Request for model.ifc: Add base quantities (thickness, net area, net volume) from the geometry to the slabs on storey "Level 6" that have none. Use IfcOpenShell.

First a look at what the model holds.

```python
import ifcopenshell
import ifcopenshell.util.element
import ifcopenshell.util.unit

model = ifcopenshell.open("model.ifc")
print(model.schema)
for unit_type in ("LENGTHUNIT", "AREAUNIT", "VOLUMEUNIT"):
    print(unit_type, ifcopenshell.util.unit.calculate_unit_scale(model, unit_type))
storey = next(s for s in model.by_type("IfcBuildingStorey") if s.Name == "Level 6")
slabs = [e for e in ifcopenshell.util.element.get_decomposition(storey) if e.is_a("IfcSlab")]
for e in sorted(slabs, key=lambda e: e.id()):
    print(e.id(), e.is_a(), e.Name, list(ifcopenshell.util.element.get_psets(e, qtos_only=True)), sep=" | ")
```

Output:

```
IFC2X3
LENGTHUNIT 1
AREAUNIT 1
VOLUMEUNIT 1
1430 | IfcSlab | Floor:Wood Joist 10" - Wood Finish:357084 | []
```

```python
import ifcopenshell
import ifcopenshell.api.pset
import ifcopenshell.geom
import ifcopenshell.util.element
import ifcopenshell.util.shape
import ifcopenshell.util.unit

model = ifcopenshell.open("model.ifc")
unit_scale = ifcopenshell.util.unit.calculate_unit_scale(model)
area_scale = ifcopenshell.util.unit.calculate_unit_scale(model, "AREAUNIT")
volume_scale = ifcopenshell.util.unit.calculate_unit_scale(model, "VOLUMEUNIT")
settings = ifcopenshell.geom.settings()

storey = next(s for s in model.by_type("IfcBuildingStorey") if s.Name == "Level 6")
slabs = [e for e in ifcopenshell.util.element.get_decomposition(storey) if e.is_a("IfcSlab")]

for e in sorted(slabs, key=lambda e: e.id()):
    if ifcopenshell.util.element.get_psets(e, qtos_only=True, should_inherit=False):
        continue
    # Geometry comes back in metres, in the element's own axes.
    shape = ifcopenshell.geom.create_shape(settings, e)
    values = {
        "Width": ifcopenshell.util.shape.get_z(shape.geometry) / unit_scale,
        "NetArea": ifcopenshell.util.shape.get_footprint_area(shape.geometry) / area_scale,
        "NetVolume": ifcopenshell.util.shape.get_volume(shape.geometry) / volume_scale,
    }
    qto = ifcopenshell.api.pset.add_qto(model, product=e, name="BaseQuantities")
    ifcopenshell.api.pset.edit_qto(model, qto=qto, properties=values)
    print(e.id(), {k: round(v, 3) for k, v in values.items()})

model.write("model-out.ifc")
```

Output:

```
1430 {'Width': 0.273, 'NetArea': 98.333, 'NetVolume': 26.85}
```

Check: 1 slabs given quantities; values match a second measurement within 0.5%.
